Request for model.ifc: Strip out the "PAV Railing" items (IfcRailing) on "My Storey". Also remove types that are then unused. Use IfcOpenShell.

First a look at what the model holds.

```python
import ifcopenshell
import ifcopenshell.util.element

model = ifcopenshell.open("model.ifc")
print(model.schema)
storey = next(s for s in model.by_type("IfcBuildingStorey") if s.Name == "My Storey")
railings = [e for e in ifcopenshell.util.element.get_decomposition(storey) if e.is_a("IfcRailing")]
seen = {}
for e in railings:
    element_type = ifcopenshell.util.element.get_type(e)
    name = element_type.Name if element_type not in (None, e) else None
    seen[name] = seen.get(name, 0) + 1
for name, count in sorted(seen.items(), key=str):
    print(count, "x", name)
```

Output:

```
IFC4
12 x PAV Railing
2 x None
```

```python
import ifcopenshell
import ifcopenshell.api.root
import ifcopenshell.util.element

model = ifcopenshell.open("model.ifc")

storey = next(s for s in model.by_type("IfcBuildingStorey") if s.Name == "My Storey")
railings = [e for e in ifcopenshell.util.element.get_decomposition(storey) if e.is_a("IfcRailing")]
targets = [e for e in railings if (t := ifcopenshell.util.element.get_type(e)) not in (None, e) and t.Name == "PAV Railing"]
types = {ifcopenshell.util.element.get_type(e) for e in targets} - {None, *targets}

for e in targets:
    ifcopenshell.api.root.remove_product(model, product=e)
print(len(targets), "removed")

unused = [t for t in types if not ifcopenshell.util.element.get_types(t)]
for t in unused:
    ifcopenshell.api.root.remove_product(model, product=t)
print(len(unused), "unused types removed")

model.write("model_rev.ifc")
```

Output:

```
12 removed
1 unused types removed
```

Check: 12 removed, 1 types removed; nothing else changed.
